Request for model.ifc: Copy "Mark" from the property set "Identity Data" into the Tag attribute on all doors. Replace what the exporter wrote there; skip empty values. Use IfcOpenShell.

First a look at what the model holds.

```python
import ifcopenshell
import ifcopenshell.util.element

model = ifcopenshell.open("model.ifc")
print(model.schema)
doors = model.by_type("IfcDoor")
print(len(doors), "doors")
for e in doors[:8]:
    source = ifcopenshell.util.element.get_pset(e, "Identity Data", "Mark")
    target = e.Tag
    print(e.id(), repr(source), repr(target), sep=" | ")
```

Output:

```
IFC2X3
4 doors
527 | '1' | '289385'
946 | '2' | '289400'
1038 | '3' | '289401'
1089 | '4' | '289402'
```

```python
import ifcopenshell
import ifcopenshell.util.element

model = ifcopenshell.open("model.ifc")

count = 0
for e in model.by_type("IfcDoor"):
    value = ifcopenshell.util.element.get_pset(e, "Identity Data", "Mark")
    current = e.Tag
    if not value or not value.strip() or current == value:
        continue
    e.Tag = value
    count += 1

print(count, "doors updated")

model.write("model_rev.ifc")
```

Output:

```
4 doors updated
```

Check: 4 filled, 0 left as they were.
